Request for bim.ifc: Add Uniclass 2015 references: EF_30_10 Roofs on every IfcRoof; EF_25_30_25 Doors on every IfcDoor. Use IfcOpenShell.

First a look at what the model holds.

```python
import ifcopenshell

model = ifcopenshell.open("bim.ifc")
print(model.schema)
print("classifications:", [c.Name for c in model.by_type("IfcClassification")])
for ifc_class in ("IfcDoor", "IfcRoof", "IfcStair", "IfcWall", "IfcWindow"):
    print(ifc_class, len(model.by_type(ifc_class)))
```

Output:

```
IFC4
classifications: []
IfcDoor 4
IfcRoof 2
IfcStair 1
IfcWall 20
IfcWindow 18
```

```python
import ifcopenshell
import ifcopenshell.api.classification

model = ifcopenshell.open("bim.ifc")

system = ifcopenshell.api.classification.add_classification(model, classification="Uniclass 2015")

codes = {
    "IfcRoof": ("EF_30_10", "Roofs"),
    "IfcDoor": ("EF_25_30_25", "Doors"),
}
for ifc_class, (code, name) in codes.items():
    products = model.by_type(ifc_class)
    ifcopenshell.api.classification.add_reference(
        model, products=products, classification=system, identification=code, name=name
    )
    print(code, len(products))

model.write("bim_rev.ifc")
```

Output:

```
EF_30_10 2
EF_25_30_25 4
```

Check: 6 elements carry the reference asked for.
